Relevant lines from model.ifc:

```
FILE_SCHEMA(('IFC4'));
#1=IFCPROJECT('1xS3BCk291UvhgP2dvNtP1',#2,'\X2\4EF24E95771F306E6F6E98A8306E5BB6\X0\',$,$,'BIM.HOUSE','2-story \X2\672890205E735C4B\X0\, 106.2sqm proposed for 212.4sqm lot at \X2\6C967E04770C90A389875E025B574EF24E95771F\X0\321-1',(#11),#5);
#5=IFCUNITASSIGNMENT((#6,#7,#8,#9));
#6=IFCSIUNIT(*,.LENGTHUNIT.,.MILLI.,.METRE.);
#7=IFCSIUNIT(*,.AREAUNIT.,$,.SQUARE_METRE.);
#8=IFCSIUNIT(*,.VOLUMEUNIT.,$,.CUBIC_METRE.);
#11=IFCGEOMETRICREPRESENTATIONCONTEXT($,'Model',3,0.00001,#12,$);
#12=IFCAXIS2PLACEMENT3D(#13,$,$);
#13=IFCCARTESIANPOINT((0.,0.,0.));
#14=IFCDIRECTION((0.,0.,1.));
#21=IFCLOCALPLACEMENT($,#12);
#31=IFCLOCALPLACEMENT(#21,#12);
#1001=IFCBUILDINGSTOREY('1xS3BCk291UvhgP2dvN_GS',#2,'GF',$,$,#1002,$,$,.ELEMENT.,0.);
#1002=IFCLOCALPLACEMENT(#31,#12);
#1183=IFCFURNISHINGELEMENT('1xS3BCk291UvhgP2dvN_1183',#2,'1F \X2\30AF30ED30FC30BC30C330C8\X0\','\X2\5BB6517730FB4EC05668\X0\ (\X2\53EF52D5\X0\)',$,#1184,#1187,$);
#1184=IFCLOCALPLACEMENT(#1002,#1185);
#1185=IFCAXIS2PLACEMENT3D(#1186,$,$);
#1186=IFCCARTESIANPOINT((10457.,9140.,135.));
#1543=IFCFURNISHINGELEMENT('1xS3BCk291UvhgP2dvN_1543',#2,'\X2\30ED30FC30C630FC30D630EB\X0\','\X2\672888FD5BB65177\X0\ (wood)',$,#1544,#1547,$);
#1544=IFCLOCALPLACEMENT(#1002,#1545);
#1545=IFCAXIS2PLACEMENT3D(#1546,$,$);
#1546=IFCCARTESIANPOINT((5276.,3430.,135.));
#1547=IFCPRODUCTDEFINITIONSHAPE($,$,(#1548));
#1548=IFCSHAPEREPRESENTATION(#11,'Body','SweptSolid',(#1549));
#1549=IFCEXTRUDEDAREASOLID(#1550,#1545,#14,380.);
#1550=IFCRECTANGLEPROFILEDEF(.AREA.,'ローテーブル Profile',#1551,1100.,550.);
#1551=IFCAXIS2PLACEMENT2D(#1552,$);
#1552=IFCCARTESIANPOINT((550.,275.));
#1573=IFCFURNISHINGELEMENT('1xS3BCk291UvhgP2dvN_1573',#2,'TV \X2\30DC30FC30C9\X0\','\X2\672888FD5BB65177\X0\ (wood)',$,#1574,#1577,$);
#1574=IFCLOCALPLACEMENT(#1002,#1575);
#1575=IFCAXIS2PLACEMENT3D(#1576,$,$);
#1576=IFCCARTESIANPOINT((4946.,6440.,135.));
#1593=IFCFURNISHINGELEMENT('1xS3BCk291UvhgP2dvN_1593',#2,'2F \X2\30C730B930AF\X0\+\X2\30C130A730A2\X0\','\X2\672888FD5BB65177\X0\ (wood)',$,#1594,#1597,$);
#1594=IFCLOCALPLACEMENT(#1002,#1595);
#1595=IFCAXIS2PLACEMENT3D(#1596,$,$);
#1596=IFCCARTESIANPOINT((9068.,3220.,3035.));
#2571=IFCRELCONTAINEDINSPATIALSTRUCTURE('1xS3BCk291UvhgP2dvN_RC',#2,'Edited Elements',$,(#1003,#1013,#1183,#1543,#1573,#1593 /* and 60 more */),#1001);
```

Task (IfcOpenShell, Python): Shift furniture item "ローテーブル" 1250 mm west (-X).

```python
import ifcopenshell
import ifcopenshell.api.geometry
import ifcopenshell.util.placement

model = ifcopenshell.open("model.ifc")

item = model.by_guid("1xS3BCk291UvhgP2dvN_1543")
matrix = ifcopenshell.util.placement.get_local_placement(item.ObjectPlacement)
matrix[0, 3] -= 1250.0
ifcopenshell.api.geometry.edit_object_placement(model, product=item, matrix=matrix, is_si=False)

print(ifcopenshell.util.placement.get_local_placement(item.ObjectPlacement).round(3) + 0.0)

model.write("model_updated.ifc")
```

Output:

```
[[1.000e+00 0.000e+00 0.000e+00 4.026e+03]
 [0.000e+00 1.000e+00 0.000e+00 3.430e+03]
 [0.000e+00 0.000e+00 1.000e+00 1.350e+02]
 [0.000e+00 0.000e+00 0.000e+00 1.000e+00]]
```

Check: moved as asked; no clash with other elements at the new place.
